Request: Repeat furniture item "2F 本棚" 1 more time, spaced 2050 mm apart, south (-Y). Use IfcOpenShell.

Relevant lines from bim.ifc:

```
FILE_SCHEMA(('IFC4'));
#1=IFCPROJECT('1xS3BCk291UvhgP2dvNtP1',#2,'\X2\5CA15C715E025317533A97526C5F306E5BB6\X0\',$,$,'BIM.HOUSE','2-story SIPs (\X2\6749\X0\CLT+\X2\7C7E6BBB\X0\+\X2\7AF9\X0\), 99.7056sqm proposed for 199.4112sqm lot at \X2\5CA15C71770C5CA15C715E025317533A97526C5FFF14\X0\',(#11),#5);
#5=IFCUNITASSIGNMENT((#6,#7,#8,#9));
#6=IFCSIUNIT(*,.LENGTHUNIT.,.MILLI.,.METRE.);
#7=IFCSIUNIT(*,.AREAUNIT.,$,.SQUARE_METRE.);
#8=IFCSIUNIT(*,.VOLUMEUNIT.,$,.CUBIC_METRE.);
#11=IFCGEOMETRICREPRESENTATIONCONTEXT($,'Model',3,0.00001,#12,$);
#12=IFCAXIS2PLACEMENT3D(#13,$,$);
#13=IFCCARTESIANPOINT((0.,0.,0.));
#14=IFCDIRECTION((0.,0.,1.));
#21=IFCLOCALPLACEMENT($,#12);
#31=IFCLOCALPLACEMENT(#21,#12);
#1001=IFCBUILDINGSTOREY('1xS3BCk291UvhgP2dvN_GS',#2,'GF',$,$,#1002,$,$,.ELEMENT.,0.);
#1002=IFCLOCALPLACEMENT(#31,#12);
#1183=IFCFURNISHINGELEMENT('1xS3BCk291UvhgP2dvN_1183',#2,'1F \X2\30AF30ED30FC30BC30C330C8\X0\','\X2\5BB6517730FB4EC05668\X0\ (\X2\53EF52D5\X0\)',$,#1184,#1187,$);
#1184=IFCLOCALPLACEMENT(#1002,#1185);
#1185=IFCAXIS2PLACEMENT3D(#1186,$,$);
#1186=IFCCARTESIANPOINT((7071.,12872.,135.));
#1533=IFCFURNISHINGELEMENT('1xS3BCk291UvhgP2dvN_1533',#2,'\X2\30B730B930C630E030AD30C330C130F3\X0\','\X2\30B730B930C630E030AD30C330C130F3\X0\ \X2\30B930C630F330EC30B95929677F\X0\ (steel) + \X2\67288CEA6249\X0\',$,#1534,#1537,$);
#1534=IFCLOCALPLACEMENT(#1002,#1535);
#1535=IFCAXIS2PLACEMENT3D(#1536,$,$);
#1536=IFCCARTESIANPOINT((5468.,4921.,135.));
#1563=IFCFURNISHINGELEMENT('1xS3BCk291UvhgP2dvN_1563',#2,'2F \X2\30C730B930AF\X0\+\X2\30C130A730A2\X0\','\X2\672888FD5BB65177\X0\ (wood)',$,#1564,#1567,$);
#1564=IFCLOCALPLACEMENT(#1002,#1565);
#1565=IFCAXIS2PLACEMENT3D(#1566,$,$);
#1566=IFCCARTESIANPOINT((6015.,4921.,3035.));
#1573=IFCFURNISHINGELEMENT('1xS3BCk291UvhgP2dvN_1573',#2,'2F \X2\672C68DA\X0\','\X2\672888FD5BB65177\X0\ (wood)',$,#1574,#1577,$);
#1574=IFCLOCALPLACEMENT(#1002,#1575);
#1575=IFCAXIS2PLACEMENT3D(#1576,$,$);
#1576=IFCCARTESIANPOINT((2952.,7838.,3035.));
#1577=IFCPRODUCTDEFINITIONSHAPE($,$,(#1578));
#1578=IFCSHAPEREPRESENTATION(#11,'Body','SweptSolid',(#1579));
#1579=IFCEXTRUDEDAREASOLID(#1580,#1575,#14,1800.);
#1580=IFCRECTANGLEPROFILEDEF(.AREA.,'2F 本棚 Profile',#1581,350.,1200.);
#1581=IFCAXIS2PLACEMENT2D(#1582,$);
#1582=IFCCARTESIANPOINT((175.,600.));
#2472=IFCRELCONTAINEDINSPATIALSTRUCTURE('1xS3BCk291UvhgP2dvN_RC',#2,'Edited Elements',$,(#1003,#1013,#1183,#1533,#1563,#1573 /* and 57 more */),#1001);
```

```python
import numpy as np
import ifcopenshell
import ifcopenshell.api.geometry
import ifcopenshell.api.root
import ifcopenshell.util.element
import ifcopenshell.util.placement
import ifcopenshell.util.unit

model = ifcopenshell.open("bim.ifc")
unit_scale = ifcopenshell.util.unit.calculate_unit_scale(model)


def reuse_history(source, copy):
    """copy_class also copies each property set's owner history, people and application; keep the originals."""
    for rel in copy.IsDefinedBy:
        if rel.is_a("IfcRelDefinesByProperties") and (history := rel.RelatingPropertyDefinition.OwnerHistory):
            rel.RelatingPropertyDefinition.OwnerHistory = source.OwnerHistory
            ifcopenshell.util.element.remove_deep2(model, history)


source = model.by_guid("1xS3BCk291UvhgP2dvN_1573")
base = ifcopenshell.util.placement.get_local_placement(source.ObjectPlacement)
step = np.array([0.0, -1.0, 0.0]) * 2.05 / unit_scale

for i in range(1, 2):
    copy = ifcopenshell.api.root.copy_class(model, product=source)
    copy.Representation = ifcopenshell.util.element.copy_deep(
        model, source.Representation, exclude=["IfcGeometricRepresentationContext", "IfcRepresentationMap"]
    )
    reuse_history(source, copy)
    matrix = base.copy()
    matrix[:3, 3] += i * step
    print("added at", matrix[:3, 3].round(3) + 0.0)
    ifcopenshell.api.geometry.edit_object_placement(model, product=copy, matrix=matrix, is_si=False)

model.write("bim_updated.ifc")
```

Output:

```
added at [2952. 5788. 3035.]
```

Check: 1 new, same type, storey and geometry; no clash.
